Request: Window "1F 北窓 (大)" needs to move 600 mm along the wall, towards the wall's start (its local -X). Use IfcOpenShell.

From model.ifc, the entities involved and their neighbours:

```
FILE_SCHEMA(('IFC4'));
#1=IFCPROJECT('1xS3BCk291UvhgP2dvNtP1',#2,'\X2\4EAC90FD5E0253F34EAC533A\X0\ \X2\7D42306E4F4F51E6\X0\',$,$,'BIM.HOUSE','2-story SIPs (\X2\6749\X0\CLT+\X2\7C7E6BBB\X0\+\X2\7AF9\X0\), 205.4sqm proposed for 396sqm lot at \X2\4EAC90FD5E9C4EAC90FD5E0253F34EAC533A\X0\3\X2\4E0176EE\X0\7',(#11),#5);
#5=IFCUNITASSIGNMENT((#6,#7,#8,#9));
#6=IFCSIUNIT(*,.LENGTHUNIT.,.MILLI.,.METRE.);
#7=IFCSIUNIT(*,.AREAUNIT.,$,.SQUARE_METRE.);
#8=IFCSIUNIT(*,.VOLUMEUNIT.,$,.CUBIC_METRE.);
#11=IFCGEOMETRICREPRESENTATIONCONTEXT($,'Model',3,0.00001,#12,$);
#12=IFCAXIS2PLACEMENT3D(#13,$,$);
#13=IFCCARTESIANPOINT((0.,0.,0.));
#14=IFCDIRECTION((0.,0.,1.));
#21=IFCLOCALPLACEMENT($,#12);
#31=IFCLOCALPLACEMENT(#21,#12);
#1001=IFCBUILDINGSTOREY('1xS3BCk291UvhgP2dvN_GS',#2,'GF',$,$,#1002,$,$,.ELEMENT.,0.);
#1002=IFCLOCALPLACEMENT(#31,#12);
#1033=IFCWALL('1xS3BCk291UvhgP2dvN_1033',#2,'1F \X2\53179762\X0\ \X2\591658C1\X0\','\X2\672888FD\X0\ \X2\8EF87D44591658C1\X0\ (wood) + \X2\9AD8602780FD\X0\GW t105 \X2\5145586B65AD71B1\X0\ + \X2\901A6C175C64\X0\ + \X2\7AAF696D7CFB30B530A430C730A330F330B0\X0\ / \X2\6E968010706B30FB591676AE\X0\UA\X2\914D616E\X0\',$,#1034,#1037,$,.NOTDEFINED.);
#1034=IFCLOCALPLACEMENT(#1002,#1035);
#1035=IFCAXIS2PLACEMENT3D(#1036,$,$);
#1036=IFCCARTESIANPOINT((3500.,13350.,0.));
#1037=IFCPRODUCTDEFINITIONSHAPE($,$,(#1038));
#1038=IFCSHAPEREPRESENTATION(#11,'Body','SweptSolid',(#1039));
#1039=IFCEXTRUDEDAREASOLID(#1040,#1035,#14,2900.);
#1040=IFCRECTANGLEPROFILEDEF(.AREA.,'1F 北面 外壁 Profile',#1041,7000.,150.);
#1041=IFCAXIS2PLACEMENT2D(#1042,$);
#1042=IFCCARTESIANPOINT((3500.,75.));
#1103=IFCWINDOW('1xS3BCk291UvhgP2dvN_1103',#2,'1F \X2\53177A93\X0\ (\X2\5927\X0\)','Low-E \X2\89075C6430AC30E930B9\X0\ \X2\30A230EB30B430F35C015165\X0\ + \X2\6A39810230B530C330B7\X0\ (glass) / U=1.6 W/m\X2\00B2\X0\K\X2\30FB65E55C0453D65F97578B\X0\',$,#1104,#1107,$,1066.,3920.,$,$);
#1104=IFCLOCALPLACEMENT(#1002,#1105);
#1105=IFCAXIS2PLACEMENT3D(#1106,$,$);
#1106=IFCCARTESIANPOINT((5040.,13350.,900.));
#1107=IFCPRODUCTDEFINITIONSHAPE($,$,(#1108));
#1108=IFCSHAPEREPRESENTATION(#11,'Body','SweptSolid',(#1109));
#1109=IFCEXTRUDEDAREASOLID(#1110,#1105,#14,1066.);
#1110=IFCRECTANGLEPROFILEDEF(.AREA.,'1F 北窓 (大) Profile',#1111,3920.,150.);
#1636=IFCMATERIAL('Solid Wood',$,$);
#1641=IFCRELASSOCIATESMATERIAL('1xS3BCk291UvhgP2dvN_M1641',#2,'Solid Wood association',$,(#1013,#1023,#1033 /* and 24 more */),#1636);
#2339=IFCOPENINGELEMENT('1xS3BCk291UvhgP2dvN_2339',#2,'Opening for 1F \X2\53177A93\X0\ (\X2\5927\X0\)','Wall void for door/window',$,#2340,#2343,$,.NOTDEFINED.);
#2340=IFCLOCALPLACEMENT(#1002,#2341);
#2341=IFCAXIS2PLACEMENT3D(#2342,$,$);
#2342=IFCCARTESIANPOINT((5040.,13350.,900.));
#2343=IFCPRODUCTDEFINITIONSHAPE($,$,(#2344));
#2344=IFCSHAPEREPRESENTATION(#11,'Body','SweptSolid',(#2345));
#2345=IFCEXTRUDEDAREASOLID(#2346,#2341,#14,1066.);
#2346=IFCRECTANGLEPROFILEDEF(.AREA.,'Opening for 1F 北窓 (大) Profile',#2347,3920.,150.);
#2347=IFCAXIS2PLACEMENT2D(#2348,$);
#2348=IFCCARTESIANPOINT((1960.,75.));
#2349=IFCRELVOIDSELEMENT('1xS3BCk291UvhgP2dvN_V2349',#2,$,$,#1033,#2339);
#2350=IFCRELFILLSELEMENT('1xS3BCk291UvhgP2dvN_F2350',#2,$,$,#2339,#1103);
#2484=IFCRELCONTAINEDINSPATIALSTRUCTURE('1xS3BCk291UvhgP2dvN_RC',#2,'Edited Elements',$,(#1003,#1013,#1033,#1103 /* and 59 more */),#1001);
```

```python
import ifcopenshell
import ifcopenshell.api.geometry
import ifcopenshell.util.placement
import ifcopenshell.util.unit

model = ifcopenshell.open("model.ifc")
unit_scale = ifcopenshell.util.unit.calculate_unit_scale(model)

window = model.by_id(1103)
opening = window.FillsVoids[0].RelatingOpeningElement
wall = opening.VoidsElements[0].RelatingBuildingElement

wall_matrix = ifcopenshell.util.placement.get_local_placement(wall.ObjectPlacement)
shift = wall_matrix[:3, 0] * -0.6 / unit_scale
before = ifcopenshell.util.placement.get_local_placement(window.ObjectPlacement)[:3, 3].copy()

# The window is not placed relative to its opening, so move both.
for product in (opening, window):
    matrix = ifcopenshell.util.placement.get_local_placement(product.ObjectPlacement)
    matrix[:3, 3] += shift
    ifcopenshell.api.geometry.edit_object_placement(model, product=product, matrix=matrix, is_si=False)

after = ifcopenshell.util.placement.get_local_placement(window.ObjectPlacement)[:3, 3]
print("window moved by", (after - before).round(3) + 0.0)

model.write("model_v2.ifc")
```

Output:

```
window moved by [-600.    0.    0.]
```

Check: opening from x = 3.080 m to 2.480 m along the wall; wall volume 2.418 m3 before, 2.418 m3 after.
